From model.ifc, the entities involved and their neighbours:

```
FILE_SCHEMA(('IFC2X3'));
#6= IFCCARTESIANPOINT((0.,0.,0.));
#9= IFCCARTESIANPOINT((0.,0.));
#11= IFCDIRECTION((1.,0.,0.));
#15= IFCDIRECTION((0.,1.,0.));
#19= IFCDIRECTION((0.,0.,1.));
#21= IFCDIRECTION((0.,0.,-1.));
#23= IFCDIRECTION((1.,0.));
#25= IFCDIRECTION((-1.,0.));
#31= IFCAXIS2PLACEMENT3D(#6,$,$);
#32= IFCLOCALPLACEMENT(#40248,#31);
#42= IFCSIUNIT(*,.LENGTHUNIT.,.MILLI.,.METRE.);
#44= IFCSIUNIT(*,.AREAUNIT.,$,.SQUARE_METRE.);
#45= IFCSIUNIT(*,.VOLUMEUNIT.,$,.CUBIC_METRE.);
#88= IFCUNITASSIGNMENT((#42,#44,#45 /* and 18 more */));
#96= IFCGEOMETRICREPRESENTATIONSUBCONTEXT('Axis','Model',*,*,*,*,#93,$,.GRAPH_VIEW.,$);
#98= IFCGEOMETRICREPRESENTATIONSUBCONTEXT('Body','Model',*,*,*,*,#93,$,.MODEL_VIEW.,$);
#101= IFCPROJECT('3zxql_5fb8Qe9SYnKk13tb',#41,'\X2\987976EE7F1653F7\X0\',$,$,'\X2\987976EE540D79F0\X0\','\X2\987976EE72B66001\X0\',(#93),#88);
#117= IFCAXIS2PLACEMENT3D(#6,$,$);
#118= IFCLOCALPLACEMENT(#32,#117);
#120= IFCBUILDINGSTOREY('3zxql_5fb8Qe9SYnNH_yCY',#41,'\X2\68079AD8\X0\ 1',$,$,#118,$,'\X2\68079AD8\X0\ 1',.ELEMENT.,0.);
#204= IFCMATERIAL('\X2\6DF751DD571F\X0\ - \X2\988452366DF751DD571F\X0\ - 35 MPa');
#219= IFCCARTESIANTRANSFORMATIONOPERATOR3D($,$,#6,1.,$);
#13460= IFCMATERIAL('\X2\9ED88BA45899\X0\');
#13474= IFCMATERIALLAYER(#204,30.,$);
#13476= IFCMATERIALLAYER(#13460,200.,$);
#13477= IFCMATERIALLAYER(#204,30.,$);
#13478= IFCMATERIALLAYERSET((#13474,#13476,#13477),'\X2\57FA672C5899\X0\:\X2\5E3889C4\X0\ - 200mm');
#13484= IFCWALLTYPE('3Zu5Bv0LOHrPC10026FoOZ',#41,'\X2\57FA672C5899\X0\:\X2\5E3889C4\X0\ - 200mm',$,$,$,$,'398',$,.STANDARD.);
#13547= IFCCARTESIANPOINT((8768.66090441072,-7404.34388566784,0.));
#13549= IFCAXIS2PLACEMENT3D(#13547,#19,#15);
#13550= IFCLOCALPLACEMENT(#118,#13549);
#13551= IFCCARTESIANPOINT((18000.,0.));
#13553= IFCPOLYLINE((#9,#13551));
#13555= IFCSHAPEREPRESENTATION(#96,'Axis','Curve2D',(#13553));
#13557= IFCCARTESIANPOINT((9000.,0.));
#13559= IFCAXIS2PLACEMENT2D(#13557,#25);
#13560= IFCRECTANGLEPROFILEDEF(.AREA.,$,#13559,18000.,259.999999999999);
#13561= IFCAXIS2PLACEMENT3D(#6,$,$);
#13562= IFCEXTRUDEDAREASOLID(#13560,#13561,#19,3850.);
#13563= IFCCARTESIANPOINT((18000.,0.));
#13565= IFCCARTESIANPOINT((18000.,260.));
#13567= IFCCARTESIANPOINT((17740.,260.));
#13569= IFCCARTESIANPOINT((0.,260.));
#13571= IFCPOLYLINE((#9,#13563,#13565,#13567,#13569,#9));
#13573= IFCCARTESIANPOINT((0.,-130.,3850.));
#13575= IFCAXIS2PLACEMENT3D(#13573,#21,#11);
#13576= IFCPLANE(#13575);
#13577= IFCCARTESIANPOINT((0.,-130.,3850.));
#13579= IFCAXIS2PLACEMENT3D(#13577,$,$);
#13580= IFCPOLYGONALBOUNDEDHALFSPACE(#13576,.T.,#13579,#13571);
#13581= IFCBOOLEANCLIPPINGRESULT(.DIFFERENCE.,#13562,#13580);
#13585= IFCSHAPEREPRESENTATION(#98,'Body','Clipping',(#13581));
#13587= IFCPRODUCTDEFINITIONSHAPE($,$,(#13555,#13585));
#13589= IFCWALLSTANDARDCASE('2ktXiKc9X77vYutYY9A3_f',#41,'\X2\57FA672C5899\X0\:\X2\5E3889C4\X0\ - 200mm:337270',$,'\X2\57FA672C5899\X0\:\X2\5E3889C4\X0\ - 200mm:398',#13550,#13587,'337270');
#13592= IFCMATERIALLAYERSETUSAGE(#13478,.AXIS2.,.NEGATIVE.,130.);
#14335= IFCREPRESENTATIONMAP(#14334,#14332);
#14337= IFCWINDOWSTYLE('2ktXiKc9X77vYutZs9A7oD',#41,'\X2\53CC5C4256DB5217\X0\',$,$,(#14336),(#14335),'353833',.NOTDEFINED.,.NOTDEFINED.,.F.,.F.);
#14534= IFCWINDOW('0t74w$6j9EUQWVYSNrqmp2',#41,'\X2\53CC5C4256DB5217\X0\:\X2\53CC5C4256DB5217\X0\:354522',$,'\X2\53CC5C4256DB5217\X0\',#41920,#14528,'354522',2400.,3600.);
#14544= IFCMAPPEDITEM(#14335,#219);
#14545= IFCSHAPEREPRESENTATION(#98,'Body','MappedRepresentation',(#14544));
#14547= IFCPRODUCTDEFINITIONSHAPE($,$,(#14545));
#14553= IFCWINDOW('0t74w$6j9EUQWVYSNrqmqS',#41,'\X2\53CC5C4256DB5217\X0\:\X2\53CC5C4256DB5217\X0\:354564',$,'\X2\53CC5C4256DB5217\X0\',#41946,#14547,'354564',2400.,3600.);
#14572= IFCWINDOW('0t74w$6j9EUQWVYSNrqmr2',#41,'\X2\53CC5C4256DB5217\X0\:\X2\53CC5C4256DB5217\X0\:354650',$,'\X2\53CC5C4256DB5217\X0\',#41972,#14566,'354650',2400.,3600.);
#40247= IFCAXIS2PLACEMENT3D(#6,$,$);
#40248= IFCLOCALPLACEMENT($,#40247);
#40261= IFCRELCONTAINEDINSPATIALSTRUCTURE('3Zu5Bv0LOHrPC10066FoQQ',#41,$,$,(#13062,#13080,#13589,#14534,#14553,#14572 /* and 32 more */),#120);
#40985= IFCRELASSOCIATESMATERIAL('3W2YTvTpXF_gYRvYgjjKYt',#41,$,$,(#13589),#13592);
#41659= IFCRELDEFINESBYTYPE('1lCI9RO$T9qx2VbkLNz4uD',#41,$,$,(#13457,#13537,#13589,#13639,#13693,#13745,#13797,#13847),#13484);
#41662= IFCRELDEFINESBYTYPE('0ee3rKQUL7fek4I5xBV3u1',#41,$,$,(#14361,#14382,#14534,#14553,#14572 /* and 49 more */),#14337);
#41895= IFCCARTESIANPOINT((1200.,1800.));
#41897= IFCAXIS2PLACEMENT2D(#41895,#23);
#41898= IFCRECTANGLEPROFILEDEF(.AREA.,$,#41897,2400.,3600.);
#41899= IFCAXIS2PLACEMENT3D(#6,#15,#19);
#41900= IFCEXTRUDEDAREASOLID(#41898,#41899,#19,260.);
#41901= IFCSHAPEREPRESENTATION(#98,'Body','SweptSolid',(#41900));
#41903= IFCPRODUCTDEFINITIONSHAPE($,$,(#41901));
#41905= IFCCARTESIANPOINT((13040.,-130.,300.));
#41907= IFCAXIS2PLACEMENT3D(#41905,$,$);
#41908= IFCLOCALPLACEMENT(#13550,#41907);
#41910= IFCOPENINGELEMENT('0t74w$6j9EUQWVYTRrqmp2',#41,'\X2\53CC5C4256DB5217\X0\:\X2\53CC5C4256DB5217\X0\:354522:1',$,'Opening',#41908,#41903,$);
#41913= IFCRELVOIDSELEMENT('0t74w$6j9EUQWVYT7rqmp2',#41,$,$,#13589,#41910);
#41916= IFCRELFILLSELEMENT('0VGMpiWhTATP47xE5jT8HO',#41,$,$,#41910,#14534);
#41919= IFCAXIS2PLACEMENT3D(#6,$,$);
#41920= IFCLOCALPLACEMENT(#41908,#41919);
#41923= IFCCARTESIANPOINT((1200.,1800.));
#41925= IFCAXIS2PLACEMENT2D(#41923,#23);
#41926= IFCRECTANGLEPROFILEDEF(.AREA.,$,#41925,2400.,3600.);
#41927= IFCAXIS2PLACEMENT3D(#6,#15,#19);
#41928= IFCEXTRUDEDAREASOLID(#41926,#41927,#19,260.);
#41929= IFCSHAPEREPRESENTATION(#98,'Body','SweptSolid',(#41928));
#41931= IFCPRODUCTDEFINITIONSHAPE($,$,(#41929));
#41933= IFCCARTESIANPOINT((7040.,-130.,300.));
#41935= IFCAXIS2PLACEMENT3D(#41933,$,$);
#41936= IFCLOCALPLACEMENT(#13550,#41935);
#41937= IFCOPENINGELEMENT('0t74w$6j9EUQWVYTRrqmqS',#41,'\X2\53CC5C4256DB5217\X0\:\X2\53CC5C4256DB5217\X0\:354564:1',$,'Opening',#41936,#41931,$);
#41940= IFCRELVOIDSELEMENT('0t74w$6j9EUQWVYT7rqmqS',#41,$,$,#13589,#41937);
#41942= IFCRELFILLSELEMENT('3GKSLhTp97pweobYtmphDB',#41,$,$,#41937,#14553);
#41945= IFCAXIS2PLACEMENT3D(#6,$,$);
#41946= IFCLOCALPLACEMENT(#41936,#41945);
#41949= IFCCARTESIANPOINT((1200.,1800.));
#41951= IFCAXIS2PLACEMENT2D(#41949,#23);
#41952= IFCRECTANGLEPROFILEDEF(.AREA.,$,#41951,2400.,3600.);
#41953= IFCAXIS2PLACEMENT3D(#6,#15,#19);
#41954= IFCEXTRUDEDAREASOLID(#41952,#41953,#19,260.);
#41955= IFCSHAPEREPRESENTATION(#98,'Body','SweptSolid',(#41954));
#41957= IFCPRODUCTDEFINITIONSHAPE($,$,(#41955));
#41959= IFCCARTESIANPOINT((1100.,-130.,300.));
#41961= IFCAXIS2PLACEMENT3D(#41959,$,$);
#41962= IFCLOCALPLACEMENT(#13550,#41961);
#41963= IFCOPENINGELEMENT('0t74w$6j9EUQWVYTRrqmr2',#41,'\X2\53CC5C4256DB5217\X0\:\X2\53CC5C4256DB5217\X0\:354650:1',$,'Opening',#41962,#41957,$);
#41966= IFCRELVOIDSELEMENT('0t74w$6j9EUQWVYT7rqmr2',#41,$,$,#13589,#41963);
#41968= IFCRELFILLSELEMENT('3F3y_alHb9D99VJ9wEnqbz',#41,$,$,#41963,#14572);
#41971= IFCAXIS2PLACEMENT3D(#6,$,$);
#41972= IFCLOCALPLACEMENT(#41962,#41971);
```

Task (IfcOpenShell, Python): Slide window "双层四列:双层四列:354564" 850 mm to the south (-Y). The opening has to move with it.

```python
import ifcopenshell
import ifcopenshell.api.geometry
import ifcopenshell.util.placement

model = ifcopenshell.open("model.ifc")

window = model.by_guid("0t74w$6j9EUQWVYSNrqmqS")
opening = window.FillsVoids[0].RelatingOpeningElement
wall = opening.VoidsElements[0].RelatingBuildingElement

wall_matrix = ifcopenshell.util.placement.get_local_placement(wall.ObjectPlacement)
shift = wall_matrix[:3, 0] * -850.0
before = ifcopenshell.util.placement.get_local_placement(window.ObjectPlacement)[:3, 3].copy()

# The window is placed relative to its opening, so it follows when the opening moves.
matrix = ifcopenshell.util.placement.get_local_placement(opening.ObjectPlacement)
matrix[:3, 3] += shift
ifcopenshell.api.geometry.edit_object_placement(
    model, product=opening, matrix=matrix, is_si=False, should_transform_children=True
)

after = ifcopenshell.util.placement.get_local_placement(window.ObjectPlacement)[:3, 3]
print("window moved by", (after - before).round(3) + 0.0)

model.write("model_v2.ifc")
```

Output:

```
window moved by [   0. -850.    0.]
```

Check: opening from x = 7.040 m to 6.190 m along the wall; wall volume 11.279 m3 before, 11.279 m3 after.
